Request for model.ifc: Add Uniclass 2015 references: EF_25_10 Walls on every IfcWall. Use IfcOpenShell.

First a look at what the model holds.

```python
import ifcopenshell

model = ifcopenshell.open("model.ifc")
print(model.schema)
print("classifications:", [c.Name for c in model.by_type("IfcClassification")])
for ifc_class in ("IfcDoor", "IfcRoof", "IfcStair", "IfcWall", "IfcWindow"):
    print(ifc_class, len(model.by_type(ifc_class)))
```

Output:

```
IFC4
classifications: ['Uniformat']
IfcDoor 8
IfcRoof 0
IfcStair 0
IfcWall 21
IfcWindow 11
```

```python
import ifcopenshell
import ifcopenshell.api.classification

model = ifcopenshell.open("model.ifc")

system = ifcopenshell.api.classification.add_classification(model, classification="Uniclass 2015")

codes = {
    "IfcWall": ("EF_25_10", "Walls"),
}
for ifc_class, (code, name) in codes.items():
    products = model.by_type(ifc_class)
    ifcopenshell.api.classification.add_reference(
        model, products=products, classification=system, identification=code, name=name
    )
    print(code, len(products))

model.write("model_edited.ifc")
```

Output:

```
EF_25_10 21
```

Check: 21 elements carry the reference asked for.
